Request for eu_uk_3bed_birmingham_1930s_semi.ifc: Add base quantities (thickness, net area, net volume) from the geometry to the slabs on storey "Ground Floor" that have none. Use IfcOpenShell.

First a look at what the model holds.

```python
import ifcopenshell
import ifcopenshell.util.element
import ifcopenshell.util.unit

model = ifcopenshell.open("eu_uk_3bed_birmingham_1930s_semi.ifc")
print(model.schema)
for unit_type in ("LENGTHUNIT", "AREAUNIT", "VOLUMEUNIT"):
    print(unit_type, ifcopenshell.util.unit.calculate_unit_scale(model, unit_type))
storey = next(s for s in model.by_type("IfcBuildingStorey") if s.Name == "Ground Floor")
slabs = [e for e in ifcopenshell.util.element.get_decomposition(storey) if e.is_a("IfcSlab")]
for e in sorted(slabs, key=lambda e: e.id()):
    print(e.id(), e.is_a(), e.Name, list(ifcopenshell.util.element.get_psets(e, qtos_only=True)), sep=" | ")
```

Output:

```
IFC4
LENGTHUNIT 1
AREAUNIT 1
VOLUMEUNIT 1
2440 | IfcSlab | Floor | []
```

```python
import ifcopenshell
import ifcopenshell.api.pset
import ifcopenshell.geom
import ifcopenshell.util.element
import ifcopenshell.util.shape
import ifcopenshell.util.unit

model = ifcopenshell.open("eu_uk_3bed_birmingham_1930s_semi.ifc")
unit_scale = ifcopenshell.util.unit.calculate_unit_scale(model)
area_scale = ifcopenshell.util.unit.calculate_unit_scale(model, "AREAUNIT")
volume_scale = ifcopenshell.util.unit.calculate_unit_scale(model, "VOLUMEUNIT")
settings = ifcopenshell.geom.settings()

storey = next(s for s in model.by_type("IfcBuildingStorey") if s.Name == "Ground Floor")
slabs = [e for e in ifcopenshell.util.element.get_decomposition(storey) if e.is_a("IfcSlab")]

for e in sorted(slabs, key=lambda e: e.id()):
    if ifcopenshell.util.element.get_psets(e, qtos_only=True, should_inherit=False):
        continue
    # Geometry comes back in metres, in the element's own axes.
    shape = ifcopenshell.geom.create_shape(settings, e)
    values = {
        "Width": ifcopenshell.util.shape.get_z(shape.geometry) / unit_scale,
        "NetArea": ifcopenshell.util.shape.get_footprint_area(shape.geometry) / area_scale,
        "NetVolume": ifcopenshell.util.shape.get_volume(shape.geometry) / volume_scale,
    }
    qto = ifcopenshell.api.pset.add_qto(model, product=e, name="Qto_SlabBaseQuantities")
    ifcopenshell.api.pset.edit_qto(model, qto=qto, properties=values)
    print(e.id(), {k: round(v, 3) for k, v in values.items()})

model.write("eu_uk_3bed_birmingham_1930s_semi_updated.ifc")
```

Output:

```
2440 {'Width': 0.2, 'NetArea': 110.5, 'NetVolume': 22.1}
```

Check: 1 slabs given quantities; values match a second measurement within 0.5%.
